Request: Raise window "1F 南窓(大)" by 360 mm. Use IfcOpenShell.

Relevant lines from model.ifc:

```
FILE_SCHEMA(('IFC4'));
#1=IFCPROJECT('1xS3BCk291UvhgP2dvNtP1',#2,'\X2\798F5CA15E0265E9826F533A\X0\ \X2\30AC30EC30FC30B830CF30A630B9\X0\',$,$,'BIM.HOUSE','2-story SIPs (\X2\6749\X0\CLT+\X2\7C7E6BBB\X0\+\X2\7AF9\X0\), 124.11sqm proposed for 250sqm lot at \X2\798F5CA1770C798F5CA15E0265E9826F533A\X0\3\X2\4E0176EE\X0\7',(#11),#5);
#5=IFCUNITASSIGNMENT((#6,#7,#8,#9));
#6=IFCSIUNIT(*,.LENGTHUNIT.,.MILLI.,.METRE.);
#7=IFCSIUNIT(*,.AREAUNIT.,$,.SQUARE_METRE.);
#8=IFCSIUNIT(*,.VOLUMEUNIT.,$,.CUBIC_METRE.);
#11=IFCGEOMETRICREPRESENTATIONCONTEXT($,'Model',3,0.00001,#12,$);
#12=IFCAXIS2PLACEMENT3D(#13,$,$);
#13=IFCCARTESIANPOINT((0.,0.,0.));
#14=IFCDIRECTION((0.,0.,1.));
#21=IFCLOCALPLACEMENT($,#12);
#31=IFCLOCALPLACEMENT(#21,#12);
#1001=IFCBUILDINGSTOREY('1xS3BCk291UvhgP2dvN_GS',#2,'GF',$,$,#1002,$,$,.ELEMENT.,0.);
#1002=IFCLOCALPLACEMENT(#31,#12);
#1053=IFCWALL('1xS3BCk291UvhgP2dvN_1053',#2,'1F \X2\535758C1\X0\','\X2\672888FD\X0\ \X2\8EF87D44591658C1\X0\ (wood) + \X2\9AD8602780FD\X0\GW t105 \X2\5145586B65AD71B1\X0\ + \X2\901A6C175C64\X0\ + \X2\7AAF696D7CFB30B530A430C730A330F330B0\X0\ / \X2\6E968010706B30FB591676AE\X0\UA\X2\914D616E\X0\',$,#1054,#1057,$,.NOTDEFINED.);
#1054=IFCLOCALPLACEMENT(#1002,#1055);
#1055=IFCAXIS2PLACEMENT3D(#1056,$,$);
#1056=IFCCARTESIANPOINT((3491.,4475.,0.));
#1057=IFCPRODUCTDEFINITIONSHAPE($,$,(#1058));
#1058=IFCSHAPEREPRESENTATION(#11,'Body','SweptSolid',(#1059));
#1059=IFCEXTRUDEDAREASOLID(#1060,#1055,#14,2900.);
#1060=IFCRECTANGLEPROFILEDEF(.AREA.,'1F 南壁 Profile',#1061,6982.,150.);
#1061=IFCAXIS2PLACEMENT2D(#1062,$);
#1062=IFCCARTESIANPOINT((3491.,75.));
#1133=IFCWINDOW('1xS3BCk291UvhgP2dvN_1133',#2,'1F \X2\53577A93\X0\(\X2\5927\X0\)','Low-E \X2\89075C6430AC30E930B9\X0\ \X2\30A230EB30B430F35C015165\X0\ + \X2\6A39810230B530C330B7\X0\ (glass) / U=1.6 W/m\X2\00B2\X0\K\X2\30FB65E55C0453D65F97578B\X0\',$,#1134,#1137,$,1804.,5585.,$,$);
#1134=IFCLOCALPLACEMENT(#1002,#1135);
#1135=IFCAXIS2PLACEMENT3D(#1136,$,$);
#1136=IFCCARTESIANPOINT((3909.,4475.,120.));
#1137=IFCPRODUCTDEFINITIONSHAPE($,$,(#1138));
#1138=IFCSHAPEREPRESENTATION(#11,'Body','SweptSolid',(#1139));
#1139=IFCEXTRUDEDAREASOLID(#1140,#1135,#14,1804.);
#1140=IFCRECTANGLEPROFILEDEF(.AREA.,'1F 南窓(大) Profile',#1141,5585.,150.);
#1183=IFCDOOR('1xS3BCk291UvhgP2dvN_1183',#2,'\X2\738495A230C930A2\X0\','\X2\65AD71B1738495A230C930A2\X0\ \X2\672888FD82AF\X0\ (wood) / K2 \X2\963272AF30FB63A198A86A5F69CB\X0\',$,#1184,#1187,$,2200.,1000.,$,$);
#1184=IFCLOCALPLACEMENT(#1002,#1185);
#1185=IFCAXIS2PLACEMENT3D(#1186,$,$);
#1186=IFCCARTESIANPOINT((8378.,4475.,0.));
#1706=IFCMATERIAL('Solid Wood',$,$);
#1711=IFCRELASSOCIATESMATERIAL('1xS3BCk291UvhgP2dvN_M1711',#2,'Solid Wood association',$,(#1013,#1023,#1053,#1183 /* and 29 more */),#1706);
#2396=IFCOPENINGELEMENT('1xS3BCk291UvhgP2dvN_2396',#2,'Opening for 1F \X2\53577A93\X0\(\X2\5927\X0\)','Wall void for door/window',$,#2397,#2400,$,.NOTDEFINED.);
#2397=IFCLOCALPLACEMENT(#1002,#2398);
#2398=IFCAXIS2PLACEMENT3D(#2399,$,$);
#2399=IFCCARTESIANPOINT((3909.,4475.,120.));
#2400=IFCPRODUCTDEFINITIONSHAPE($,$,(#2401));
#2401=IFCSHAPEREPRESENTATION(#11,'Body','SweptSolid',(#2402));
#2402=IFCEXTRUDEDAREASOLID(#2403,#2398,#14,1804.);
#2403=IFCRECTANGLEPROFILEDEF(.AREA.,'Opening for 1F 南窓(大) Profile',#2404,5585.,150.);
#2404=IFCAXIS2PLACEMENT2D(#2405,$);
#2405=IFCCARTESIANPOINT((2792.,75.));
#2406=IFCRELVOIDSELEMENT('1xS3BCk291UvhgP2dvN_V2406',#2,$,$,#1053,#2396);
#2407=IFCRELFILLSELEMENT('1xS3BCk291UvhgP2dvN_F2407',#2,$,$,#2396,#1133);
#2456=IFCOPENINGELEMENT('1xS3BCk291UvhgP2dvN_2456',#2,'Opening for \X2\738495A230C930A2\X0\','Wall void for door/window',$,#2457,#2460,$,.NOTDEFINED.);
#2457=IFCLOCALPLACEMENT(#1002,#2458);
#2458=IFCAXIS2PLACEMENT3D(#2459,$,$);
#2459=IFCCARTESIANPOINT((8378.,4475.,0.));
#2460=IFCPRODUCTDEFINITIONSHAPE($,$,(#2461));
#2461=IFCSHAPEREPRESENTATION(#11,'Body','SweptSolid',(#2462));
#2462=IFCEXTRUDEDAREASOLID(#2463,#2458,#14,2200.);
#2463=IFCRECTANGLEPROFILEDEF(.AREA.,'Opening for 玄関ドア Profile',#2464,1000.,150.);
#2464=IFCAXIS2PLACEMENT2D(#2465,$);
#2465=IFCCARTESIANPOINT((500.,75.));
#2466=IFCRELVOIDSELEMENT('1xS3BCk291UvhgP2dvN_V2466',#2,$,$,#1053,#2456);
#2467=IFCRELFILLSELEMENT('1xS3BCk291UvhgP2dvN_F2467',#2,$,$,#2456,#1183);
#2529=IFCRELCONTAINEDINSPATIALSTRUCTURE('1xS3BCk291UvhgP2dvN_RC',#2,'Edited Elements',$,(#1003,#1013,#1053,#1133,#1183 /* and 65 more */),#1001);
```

```python
import numpy as np
import ifcopenshell
import ifcopenshell.api.geometry
import ifcopenshell.util.placement
import ifcopenshell.util.unit

model = ifcopenshell.open("model.ifc")
unit_scale = ifcopenshell.util.unit.calculate_unit_scale(model)

window = model.by_guid("1xS3BCk291UvhgP2dvN_1133")
opening = window.FillsVoids[0].RelatingOpeningElement
dz = 0.36 / unit_scale

shift = np.array([0.0, 0.0, dz])
# The window is not placed relative to its opening, so move both.
for product in (opening, window):
    matrix = ifcopenshell.util.placement.get_local_placement(product.ObjectPlacement)
    matrix[:3, 3] += shift
    ifcopenshell.api.geometry.edit_object_placement(model, product=product, matrix=matrix, is_si=False)

print(f"moved by {dz * unit_scale:+.3f} m")

model.write("model_v2.ifc")
```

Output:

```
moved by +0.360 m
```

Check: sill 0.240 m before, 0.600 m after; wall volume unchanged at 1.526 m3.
